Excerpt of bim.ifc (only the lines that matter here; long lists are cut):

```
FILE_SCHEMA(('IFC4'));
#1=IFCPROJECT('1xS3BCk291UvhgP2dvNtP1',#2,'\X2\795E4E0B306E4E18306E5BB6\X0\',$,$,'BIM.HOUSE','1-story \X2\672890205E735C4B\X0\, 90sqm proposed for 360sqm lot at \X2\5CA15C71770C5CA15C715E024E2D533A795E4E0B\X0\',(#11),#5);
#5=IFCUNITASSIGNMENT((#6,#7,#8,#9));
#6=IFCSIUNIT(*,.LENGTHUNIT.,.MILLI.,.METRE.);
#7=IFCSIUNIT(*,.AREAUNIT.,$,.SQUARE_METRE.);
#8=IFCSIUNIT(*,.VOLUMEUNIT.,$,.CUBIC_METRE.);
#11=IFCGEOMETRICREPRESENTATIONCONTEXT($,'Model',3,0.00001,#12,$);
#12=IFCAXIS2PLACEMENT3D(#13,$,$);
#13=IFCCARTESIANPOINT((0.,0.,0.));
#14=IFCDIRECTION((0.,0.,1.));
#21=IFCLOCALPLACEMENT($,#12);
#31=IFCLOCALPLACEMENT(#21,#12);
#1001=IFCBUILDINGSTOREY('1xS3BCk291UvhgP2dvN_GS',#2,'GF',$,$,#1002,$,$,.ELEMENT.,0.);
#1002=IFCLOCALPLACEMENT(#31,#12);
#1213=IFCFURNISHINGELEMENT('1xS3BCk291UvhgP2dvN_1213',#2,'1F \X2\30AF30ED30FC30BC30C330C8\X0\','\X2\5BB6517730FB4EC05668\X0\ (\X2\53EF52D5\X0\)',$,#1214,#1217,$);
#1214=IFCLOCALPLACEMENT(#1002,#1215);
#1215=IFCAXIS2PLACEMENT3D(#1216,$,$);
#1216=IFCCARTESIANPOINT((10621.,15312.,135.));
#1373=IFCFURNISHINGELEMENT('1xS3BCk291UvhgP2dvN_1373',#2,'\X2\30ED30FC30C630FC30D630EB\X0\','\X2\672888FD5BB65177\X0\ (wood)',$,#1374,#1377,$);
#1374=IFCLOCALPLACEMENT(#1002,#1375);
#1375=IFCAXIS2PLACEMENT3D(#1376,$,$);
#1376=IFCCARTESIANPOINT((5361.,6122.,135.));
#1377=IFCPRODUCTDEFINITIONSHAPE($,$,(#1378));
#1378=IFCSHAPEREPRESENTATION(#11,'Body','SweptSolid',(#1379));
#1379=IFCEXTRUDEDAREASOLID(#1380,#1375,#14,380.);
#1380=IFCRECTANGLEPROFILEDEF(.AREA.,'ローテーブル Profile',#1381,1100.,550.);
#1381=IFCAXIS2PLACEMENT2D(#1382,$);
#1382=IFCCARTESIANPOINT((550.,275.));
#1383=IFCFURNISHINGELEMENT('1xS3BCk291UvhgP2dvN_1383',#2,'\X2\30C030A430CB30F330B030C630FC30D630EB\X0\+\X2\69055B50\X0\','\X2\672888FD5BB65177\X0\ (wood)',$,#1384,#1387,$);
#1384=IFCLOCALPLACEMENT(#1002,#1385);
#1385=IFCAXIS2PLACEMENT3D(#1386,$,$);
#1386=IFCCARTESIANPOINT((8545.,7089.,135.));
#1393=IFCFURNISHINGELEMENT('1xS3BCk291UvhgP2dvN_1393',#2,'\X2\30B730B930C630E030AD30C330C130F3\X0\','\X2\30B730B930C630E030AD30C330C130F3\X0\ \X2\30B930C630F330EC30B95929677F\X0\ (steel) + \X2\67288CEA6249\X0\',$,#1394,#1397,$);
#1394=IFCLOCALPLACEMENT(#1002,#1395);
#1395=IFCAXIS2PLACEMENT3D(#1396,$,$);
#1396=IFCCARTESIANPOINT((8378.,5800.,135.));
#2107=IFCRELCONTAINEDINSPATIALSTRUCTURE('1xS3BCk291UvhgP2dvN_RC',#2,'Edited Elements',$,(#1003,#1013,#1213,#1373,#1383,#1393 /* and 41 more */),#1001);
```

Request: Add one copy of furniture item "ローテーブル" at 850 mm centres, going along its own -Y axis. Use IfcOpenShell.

```python
import ifcopenshell
import ifcopenshell.api.geometry
import ifcopenshell.api.root
import ifcopenshell.util.element
import ifcopenshell.util.placement
import ifcopenshell.util.unit

model = ifcopenshell.open("bim.ifc")
unit_scale = ifcopenshell.util.unit.calculate_unit_scale(model)


def reuse_history(source, copy):
    """copy_class also copies each property set's owner history, people and application; keep the originals."""
    for rel in copy.IsDefinedBy:
        if rel.is_a("IfcRelDefinesByProperties") and (history := rel.RelatingPropertyDefinition.OwnerHistory):
            rel.RelatingPropertyDefinition.OwnerHistory = source.OwnerHistory
            ifcopenshell.util.element.remove_deep2(model, history)


source = model.by_id(1373)
base = ifcopenshell.util.placement.get_local_placement(source.ObjectPlacement)
step = -base[:3, 1] * 0.85 / unit_scale

for i in range(1, 2):
    copy = ifcopenshell.api.root.copy_class(model, product=source)
    copy.Representation = ifcopenshell.util.element.copy_deep(
        model, source.Representation, exclude=["IfcGeometricRepresentationContext", "IfcRepresentationMap"]
    )
    reuse_history(source, copy)
    matrix = base.copy()
    matrix[:3, 3] += i * step
    print("added at", matrix[:3, 3].round(3) + 0.0)
    ifcopenshell.api.geometry.edit_object_placement(model, product=copy, matrix=matrix, is_si=False)

model.write("bim_rev.ifc")
```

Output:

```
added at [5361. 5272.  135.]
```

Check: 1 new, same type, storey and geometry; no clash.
